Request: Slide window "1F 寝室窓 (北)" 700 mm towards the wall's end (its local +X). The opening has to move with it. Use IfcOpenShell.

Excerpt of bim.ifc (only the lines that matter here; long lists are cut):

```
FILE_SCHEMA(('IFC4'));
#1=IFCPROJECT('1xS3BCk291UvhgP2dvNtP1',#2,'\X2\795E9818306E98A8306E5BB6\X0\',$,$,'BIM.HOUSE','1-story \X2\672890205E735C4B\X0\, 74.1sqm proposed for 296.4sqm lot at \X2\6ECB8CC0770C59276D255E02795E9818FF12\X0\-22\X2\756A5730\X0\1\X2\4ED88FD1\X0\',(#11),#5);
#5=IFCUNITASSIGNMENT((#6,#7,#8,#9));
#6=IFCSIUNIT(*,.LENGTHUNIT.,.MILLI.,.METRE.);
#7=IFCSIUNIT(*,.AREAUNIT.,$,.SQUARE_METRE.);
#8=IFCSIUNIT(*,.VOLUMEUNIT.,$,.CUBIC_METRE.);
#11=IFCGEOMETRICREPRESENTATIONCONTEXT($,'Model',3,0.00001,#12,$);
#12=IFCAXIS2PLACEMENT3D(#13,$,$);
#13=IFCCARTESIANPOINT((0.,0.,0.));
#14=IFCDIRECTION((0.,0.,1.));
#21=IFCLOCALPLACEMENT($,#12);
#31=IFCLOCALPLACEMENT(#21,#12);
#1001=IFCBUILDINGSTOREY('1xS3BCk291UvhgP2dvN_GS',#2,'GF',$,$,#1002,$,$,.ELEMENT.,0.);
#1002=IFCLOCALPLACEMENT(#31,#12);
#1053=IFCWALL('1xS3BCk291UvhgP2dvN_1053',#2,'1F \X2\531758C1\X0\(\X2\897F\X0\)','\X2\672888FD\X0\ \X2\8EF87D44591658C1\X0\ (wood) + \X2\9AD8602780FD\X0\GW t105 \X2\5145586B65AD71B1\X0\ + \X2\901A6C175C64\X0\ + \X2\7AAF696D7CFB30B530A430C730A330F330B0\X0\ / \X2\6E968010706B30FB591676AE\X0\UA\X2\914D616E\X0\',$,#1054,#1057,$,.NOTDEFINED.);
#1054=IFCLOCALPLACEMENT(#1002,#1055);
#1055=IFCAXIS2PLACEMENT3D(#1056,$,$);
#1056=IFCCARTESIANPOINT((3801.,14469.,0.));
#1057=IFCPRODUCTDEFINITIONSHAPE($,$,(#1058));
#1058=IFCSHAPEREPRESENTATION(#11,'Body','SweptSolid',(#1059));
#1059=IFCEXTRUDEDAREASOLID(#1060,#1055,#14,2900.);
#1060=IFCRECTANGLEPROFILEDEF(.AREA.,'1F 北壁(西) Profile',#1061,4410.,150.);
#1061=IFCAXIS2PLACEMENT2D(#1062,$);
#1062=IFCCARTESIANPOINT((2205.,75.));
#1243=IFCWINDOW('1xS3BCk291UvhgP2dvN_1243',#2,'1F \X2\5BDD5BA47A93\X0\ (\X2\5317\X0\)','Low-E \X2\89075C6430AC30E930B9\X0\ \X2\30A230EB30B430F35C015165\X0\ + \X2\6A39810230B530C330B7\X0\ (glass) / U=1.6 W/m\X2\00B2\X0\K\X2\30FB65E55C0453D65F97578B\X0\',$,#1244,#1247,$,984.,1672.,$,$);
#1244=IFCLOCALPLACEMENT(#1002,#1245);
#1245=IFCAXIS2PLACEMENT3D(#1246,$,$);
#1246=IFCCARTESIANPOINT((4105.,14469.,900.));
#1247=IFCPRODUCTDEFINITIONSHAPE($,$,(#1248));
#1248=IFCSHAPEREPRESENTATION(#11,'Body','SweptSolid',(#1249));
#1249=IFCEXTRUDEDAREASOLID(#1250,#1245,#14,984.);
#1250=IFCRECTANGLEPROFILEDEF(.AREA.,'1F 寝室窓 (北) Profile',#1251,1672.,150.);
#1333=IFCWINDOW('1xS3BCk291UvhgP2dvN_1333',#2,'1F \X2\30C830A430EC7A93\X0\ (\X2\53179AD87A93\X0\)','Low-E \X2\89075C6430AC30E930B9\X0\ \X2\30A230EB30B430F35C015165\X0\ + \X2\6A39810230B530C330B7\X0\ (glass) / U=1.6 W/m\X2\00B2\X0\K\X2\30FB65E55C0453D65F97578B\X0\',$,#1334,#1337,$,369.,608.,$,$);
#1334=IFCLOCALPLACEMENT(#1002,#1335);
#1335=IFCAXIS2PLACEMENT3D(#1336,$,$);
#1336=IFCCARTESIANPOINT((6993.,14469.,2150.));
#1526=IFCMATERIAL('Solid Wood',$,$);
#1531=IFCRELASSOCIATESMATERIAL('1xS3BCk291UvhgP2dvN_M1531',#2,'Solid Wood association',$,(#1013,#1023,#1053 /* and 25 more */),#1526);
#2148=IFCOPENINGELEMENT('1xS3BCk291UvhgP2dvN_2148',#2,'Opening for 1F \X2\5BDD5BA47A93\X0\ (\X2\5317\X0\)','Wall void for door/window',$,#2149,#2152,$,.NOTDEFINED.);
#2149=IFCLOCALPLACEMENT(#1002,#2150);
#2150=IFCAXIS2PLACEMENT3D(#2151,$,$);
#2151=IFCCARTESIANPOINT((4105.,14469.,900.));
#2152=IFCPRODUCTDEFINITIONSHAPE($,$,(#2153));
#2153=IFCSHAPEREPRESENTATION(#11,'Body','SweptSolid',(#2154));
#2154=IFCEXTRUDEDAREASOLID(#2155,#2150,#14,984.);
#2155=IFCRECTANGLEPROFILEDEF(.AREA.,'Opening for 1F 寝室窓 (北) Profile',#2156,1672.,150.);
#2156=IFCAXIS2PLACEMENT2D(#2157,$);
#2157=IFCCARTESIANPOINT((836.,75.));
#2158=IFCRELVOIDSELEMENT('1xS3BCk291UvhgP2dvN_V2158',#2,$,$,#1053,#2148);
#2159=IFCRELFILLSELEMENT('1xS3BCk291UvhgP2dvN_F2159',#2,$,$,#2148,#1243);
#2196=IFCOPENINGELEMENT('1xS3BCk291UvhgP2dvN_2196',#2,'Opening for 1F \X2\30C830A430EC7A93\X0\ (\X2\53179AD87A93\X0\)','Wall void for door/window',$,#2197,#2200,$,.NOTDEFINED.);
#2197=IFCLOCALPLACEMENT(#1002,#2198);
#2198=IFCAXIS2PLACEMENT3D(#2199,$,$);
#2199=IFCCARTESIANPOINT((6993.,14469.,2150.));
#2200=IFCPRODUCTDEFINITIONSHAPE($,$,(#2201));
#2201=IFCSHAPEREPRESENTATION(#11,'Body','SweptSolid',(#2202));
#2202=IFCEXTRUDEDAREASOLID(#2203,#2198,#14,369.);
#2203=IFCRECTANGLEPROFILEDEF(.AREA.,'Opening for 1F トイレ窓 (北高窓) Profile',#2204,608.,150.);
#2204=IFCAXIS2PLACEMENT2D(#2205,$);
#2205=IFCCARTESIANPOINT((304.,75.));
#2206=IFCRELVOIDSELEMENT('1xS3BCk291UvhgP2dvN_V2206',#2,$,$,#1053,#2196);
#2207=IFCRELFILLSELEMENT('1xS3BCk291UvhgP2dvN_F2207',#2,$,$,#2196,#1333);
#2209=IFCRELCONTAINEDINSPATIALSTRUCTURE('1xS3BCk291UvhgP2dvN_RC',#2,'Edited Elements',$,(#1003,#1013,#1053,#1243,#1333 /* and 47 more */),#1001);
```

```python
import ifcopenshell
import ifcopenshell.api.geometry
import ifcopenshell.util.placement
import ifcopenshell.util.unit

model = ifcopenshell.open("bim.ifc")
unit_scale = ifcopenshell.util.unit.calculate_unit_scale(model)

window = model.by_guid("1xS3BCk291UvhgP2dvN_1243")
opening = window.FillsVoids[0].RelatingOpeningElement
wall = opening.VoidsElements[0].RelatingBuildingElement

wall_matrix = ifcopenshell.util.placement.get_local_placement(wall.ObjectPlacement)
shift = wall_matrix[:3, 0] * 0.7 / unit_scale
before = ifcopenshell.util.placement.get_local_placement(window.ObjectPlacement)[:3, 3].copy()

# The window is not placed relative to its opening, so move both.
for product in (opening, window):
    matrix = ifcopenshell.util.placement.get_local_placement(product.ObjectPlacement)
    matrix[:3, 3] += shift
    ifcopenshell.api.geometry.edit_object_placement(model, product=product, matrix=matrix, is_si=False)

after = ifcopenshell.util.placement.get_local_placement(window.ObjectPlacement)[:3, 3]
print("window moved by", (after - before).round(3) + 0.0)

model.write("bim_v2.ifc")
```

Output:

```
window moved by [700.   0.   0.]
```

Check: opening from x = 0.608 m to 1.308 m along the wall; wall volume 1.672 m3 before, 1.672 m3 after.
